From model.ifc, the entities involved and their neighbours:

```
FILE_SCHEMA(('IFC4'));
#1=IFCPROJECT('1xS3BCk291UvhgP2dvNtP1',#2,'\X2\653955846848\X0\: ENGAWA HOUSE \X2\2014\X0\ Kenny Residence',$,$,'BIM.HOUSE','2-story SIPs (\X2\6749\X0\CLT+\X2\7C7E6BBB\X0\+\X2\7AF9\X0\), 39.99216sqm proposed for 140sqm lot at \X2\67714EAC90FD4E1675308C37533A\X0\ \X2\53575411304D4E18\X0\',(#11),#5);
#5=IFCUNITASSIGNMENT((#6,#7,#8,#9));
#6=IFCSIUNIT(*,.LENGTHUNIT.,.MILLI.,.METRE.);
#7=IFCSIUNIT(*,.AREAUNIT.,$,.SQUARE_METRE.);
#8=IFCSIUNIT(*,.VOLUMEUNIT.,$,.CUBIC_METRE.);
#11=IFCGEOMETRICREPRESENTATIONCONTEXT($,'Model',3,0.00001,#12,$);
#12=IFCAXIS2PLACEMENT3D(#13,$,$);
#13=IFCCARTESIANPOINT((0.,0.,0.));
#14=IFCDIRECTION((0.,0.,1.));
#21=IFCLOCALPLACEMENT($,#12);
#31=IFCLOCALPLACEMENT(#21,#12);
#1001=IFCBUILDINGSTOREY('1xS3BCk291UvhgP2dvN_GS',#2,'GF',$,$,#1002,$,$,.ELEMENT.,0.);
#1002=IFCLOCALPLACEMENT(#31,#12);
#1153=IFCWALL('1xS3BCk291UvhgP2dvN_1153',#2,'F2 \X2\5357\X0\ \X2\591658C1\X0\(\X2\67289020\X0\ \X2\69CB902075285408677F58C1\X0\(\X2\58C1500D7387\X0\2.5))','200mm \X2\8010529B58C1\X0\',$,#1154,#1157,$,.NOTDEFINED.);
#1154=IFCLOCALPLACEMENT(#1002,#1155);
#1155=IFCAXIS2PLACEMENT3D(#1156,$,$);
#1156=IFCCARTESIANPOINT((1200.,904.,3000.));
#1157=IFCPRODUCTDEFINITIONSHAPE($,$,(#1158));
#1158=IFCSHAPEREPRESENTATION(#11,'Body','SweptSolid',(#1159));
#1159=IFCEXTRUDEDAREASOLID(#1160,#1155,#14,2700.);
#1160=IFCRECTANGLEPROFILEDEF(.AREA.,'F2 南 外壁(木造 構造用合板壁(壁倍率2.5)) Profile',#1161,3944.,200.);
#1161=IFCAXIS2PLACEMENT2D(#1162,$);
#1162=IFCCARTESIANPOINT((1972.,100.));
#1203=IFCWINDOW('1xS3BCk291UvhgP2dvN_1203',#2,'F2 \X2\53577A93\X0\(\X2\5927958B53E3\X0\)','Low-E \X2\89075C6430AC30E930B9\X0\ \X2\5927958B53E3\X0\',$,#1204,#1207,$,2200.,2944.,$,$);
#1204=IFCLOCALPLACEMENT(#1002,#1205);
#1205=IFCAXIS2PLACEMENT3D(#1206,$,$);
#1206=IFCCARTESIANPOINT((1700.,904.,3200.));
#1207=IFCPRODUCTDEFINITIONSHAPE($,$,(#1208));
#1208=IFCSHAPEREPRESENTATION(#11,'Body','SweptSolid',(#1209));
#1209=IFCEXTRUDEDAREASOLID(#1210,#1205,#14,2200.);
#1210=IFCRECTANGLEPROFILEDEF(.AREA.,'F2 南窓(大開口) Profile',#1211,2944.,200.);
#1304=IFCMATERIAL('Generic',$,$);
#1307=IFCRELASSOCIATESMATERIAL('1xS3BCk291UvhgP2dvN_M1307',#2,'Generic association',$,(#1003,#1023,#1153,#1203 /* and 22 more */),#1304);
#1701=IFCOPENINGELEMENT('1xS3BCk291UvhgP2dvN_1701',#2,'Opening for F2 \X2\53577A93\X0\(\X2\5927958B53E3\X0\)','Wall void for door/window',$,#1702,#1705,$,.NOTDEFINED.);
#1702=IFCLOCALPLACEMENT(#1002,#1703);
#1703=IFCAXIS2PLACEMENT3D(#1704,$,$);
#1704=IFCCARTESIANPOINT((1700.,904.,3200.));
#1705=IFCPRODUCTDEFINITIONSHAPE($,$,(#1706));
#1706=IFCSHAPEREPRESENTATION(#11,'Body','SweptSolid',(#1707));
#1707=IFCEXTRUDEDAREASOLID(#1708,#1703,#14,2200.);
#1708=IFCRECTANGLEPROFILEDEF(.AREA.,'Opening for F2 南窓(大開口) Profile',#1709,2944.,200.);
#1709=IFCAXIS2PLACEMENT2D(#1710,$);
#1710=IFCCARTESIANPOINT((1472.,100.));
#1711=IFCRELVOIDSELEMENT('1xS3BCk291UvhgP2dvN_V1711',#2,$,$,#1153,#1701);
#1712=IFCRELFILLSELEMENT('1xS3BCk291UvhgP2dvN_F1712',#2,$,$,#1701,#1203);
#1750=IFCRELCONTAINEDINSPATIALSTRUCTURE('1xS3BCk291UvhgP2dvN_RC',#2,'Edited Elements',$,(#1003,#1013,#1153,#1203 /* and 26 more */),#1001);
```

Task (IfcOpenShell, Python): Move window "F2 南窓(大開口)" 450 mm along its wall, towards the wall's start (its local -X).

```python
import ifcopenshell
import ifcopenshell.api.geometry
import ifcopenshell.util.placement
import ifcopenshell.util.unit

model = ifcopenshell.open("model.ifc")
unit_scale = ifcopenshell.util.unit.calculate_unit_scale(model)

window = model.by_id(1203)
opening = window.FillsVoids[0].RelatingOpeningElement
wall = opening.VoidsElements[0].RelatingBuildingElement

wall_matrix = ifcopenshell.util.placement.get_local_placement(wall.ObjectPlacement)
shift = wall_matrix[:3, 0] * -0.45 / unit_scale
before = ifcopenshell.util.placement.get_local_placement(window.ObjectPlacement)[:3, 3].copy()

# The window is not placed relative to its opening, so move both.
for product in (opening, window):
    matrix = ifcopenshell.util.placement.get_local_placement(product.ObjectPlacement)
    matrix[:3, 3] += shift
    ifcopenshell.api.geometry.edit_object_placement(model, product=product, matrix=matrix, is_si=False)

after = ifcopenshell.util.placement.get_local_placement(window.ObjectPlacement)[:3, 3]
print("window moved by", (after - before).round(3) + 0.0)

model.write("model_edited.ifc")
```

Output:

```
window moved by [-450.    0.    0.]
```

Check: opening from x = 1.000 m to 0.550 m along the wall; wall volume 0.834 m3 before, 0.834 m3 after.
